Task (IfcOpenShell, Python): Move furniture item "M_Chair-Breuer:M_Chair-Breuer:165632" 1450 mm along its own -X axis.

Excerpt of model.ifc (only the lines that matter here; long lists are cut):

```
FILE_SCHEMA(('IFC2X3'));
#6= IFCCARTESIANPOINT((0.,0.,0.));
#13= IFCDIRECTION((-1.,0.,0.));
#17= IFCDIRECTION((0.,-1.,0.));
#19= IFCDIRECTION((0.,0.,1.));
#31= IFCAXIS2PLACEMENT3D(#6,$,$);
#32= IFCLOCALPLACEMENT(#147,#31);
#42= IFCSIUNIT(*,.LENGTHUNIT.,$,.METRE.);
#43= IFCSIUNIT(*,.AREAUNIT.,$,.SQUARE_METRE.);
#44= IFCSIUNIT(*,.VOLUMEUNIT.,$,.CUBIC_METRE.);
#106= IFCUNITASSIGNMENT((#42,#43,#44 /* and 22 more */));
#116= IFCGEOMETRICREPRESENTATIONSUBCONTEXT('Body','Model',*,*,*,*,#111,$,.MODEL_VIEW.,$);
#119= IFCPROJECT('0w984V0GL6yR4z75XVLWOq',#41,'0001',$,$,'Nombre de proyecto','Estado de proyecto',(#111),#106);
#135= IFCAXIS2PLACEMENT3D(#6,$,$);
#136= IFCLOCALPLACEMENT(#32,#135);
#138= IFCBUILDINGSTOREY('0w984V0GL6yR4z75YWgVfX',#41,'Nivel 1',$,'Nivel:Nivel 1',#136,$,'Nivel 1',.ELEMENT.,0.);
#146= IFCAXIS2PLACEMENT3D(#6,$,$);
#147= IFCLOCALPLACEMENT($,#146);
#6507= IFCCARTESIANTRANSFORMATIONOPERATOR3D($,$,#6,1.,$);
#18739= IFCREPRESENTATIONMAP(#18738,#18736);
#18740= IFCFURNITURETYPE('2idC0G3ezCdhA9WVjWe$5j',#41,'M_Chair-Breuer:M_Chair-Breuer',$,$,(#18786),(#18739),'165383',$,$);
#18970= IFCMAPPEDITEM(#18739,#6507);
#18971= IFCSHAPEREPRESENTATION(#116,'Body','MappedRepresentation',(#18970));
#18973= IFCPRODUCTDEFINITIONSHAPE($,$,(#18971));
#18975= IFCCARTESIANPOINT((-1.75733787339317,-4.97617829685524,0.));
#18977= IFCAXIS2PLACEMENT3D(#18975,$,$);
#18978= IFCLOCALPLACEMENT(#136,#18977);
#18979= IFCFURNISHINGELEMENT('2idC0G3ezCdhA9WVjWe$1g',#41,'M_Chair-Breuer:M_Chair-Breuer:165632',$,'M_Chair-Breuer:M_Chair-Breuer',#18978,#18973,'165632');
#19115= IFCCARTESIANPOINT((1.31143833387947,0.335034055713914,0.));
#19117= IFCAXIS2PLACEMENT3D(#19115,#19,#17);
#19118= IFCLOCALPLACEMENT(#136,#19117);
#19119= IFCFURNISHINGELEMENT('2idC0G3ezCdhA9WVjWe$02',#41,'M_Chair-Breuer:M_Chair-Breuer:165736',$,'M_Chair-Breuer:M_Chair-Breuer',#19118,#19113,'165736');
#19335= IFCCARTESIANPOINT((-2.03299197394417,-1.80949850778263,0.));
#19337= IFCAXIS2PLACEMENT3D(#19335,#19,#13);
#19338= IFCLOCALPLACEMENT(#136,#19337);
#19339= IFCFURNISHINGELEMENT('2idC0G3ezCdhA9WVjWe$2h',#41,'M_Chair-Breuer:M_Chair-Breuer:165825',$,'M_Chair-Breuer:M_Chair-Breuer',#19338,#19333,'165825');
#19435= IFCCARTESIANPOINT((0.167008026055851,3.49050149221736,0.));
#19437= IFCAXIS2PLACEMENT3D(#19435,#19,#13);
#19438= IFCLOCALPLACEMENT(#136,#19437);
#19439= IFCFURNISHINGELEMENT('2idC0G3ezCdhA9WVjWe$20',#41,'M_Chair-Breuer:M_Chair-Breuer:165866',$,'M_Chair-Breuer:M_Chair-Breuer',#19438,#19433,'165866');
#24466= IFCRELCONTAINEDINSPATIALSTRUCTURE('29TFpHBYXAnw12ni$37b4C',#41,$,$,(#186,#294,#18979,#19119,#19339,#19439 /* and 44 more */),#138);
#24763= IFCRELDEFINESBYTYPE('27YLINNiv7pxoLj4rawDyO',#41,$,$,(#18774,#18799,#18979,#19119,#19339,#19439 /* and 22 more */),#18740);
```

```python
import ifcopenshell
import ifcopenshell.api.geometry
import ifcopenshell.util.placement

model = ifcopenshell.open("model.ifc")

item = model.by_guid("2idC0G3ezCdhA9WVjWe$1g")
matrix = ifcopenshell.util.placement.get_local_placement(item.ObjectPlacement)
matrix[:3, 3] -= matrix[:3, 0] * 1.45
ifcopenshell.api.geometry.edit_object_placement(model, product=item, matrix=matrix, is_si=False)

print(ifcopenshell.util.placement.get_local_placement(item.ObjectPlacement).round(3) + 0.0)

model.write("model_v2.ifc")
```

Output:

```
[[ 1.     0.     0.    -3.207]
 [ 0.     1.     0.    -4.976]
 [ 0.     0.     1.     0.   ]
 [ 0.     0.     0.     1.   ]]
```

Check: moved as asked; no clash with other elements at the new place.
